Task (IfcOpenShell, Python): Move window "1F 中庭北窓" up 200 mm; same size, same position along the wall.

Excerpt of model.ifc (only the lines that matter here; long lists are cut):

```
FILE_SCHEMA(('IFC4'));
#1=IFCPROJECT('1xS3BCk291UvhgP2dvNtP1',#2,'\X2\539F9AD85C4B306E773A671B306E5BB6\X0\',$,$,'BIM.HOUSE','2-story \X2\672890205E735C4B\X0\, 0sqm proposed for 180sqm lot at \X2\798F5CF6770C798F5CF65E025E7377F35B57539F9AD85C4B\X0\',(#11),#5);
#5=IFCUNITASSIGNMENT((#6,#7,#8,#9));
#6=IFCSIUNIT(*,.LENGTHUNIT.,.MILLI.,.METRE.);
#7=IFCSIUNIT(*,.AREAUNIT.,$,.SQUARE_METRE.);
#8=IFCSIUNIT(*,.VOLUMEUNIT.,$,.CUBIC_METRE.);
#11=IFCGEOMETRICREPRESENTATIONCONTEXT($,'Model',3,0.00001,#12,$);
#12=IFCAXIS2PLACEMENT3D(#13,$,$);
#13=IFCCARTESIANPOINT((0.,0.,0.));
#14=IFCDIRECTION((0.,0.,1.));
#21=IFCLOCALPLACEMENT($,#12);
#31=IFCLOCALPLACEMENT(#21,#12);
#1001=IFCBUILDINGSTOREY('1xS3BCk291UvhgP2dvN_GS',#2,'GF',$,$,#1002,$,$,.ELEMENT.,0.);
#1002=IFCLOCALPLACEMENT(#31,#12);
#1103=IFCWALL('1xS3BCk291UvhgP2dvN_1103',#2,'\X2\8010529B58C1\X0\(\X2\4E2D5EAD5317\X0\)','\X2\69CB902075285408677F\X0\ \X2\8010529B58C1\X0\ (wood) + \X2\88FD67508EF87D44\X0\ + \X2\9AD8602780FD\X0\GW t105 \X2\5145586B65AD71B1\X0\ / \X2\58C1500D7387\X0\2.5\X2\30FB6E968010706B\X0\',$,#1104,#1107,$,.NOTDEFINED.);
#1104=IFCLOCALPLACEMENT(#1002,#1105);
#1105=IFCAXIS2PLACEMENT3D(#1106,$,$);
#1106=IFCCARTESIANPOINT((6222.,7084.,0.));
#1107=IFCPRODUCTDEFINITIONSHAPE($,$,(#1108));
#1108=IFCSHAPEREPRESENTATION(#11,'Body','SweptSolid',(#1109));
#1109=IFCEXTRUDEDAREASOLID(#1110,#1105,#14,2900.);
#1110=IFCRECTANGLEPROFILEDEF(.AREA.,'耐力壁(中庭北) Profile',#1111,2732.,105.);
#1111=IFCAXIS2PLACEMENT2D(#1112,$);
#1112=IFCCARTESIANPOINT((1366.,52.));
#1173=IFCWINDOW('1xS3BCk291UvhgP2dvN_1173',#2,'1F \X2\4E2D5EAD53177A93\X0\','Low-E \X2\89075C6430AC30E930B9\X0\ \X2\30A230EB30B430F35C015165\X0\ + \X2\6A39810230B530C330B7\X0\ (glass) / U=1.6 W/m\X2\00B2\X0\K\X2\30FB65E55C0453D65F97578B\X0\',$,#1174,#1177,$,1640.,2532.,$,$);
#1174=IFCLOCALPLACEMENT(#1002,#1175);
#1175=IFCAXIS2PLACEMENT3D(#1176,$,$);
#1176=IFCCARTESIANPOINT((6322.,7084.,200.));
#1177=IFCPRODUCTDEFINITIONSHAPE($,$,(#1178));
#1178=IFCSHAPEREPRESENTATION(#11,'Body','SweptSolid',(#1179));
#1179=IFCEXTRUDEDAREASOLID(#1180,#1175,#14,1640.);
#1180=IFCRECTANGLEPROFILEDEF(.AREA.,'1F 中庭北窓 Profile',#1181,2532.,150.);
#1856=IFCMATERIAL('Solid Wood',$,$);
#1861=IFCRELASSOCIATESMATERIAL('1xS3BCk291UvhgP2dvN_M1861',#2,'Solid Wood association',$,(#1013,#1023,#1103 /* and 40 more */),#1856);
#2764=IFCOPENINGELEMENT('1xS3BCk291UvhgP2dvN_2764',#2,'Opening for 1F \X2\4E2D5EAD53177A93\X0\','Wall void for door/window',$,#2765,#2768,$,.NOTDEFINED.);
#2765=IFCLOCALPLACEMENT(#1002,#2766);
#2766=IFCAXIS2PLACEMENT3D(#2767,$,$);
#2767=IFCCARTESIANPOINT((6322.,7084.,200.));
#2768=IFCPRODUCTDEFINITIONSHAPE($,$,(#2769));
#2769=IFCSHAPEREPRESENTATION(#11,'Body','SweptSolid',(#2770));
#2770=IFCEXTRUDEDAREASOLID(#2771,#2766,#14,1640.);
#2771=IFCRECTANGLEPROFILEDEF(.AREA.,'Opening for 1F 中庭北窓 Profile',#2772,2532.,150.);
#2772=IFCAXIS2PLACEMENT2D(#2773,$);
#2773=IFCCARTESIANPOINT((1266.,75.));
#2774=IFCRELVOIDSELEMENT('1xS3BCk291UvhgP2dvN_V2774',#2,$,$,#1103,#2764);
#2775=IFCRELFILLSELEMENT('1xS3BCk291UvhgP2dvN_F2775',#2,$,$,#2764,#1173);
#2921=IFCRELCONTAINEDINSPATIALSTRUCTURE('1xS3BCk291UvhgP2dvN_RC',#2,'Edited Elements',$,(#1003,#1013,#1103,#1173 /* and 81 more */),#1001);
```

```python
import numpy as np
import ifcopenshell
import ifcopenshell.api.geometry
import ifcopenshell.util.placement
import ifcopenshell.util.unit

model = ifcopenshell.open("model.ifc")
unit_scale = ifcopenshell.util.unit.calculate_unit_scale(model)

window = model.by_guid("1xS3BCk291UvhgP2dvN_1173")
opening = window.FillsVoids[0].RelatingOpeningElement
dz = 0.2 / unit_scale

shift = np.array([0.0, 0.0, dz])
# The window is not placed relative to its opening, so move both.
for product in (opening, window):
    matrix = ifcopenshell.util.placement.get_local_placement(product.ObjectPlacement)
    matrix[:3, 3] += shift
    ifcopenshell.api.geometry.edit_object_placement(model, product=product, matrix=matrix, is_si=False)

print(f"moved by {dz * unit_scale:+.3f} m")

model.write("model_edited.ifc")
```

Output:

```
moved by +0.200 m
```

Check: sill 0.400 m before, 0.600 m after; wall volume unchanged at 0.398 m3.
